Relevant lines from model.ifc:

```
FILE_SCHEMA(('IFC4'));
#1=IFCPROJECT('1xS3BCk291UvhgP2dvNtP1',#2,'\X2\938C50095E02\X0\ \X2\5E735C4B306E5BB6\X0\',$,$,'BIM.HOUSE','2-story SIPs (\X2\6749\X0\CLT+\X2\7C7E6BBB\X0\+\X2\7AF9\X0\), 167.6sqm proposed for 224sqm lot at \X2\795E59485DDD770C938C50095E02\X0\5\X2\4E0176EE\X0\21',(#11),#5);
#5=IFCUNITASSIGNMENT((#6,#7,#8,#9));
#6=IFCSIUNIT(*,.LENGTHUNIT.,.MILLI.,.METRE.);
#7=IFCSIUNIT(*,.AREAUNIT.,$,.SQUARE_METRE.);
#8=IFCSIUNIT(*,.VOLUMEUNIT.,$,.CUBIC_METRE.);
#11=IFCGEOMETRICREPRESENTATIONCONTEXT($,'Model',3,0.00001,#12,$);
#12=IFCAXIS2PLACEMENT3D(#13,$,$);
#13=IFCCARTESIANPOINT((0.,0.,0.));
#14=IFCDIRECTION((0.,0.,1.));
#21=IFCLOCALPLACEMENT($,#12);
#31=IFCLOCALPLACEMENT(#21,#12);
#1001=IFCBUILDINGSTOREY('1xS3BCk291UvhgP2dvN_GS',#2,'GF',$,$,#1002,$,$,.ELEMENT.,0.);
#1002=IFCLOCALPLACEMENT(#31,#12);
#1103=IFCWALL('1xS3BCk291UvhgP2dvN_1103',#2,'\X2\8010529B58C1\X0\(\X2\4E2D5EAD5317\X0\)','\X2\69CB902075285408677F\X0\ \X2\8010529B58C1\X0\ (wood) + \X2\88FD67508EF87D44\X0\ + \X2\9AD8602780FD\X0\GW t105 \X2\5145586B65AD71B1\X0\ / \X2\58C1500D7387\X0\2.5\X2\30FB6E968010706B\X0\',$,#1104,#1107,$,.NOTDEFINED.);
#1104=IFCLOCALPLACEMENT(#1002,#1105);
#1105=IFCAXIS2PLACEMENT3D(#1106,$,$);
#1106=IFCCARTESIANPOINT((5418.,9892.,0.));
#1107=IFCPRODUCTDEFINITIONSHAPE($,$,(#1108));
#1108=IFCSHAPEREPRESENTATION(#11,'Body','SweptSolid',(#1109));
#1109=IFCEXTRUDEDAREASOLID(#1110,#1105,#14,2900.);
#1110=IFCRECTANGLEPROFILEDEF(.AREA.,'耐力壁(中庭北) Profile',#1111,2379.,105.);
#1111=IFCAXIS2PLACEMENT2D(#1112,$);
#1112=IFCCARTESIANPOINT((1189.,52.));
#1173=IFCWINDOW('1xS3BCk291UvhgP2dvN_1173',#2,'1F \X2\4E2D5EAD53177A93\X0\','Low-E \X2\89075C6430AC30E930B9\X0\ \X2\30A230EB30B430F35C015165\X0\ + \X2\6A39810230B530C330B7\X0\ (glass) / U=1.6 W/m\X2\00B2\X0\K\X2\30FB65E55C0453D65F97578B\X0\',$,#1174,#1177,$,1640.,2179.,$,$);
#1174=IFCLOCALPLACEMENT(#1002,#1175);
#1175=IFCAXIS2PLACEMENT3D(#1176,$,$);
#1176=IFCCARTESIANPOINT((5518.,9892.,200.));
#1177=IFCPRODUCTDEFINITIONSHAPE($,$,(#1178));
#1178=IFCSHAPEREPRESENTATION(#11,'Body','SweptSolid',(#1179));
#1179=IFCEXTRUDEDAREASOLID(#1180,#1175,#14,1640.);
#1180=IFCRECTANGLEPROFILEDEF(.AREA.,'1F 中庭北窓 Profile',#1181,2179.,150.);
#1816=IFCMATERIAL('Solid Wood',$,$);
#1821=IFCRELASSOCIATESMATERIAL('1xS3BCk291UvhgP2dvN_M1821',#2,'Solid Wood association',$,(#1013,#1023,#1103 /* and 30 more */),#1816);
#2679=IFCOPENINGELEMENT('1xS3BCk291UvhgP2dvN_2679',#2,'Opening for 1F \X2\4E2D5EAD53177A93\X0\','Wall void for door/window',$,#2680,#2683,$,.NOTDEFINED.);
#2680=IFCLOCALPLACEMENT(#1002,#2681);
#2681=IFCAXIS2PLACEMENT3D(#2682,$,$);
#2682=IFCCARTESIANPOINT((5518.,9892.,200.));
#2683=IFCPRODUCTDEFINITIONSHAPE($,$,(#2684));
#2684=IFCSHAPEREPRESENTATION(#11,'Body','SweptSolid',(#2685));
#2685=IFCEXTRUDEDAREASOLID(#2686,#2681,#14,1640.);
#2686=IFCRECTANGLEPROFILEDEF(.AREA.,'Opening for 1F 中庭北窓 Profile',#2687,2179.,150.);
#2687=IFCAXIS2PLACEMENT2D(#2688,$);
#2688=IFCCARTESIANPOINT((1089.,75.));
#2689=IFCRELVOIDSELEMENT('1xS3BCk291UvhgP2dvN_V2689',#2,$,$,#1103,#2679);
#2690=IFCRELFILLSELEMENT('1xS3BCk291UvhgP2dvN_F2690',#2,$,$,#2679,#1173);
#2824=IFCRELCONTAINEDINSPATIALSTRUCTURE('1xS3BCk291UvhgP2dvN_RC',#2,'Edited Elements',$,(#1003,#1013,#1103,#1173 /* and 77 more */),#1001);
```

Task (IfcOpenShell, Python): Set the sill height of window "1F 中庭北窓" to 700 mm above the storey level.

```python
import numpy as np
import ifcopenshell
import ifcopenshell.api.geometry
import ifcopenshell.geom
import ifcopenshell.util.element
import ifcopenshell.util.placement
import ifcopenshell.util.shape
import ifcopenshell.util.unit

model = ifcopenshell.open("model.ifc")
unit_scale = ifcopenshell.util.unit.calculate_unit_scale(model)

window = model.by_id(1173)
opening = window.FillsVoids[0].RelatingOpeningElement
storey = ifcopenshell.util.element.get_container(window, ifc_class="IfcBuildingStorey")
level = ifcopenshell.util.placement.get_local_placement(storey.ObjectPlacement)[2, 3]

# The opening's origin need not be at the sill, so measure its lowest point.
shape = ifcopenshell.geom.create_shape(ifcopenshell.geom.settings(), opening)
bottom = ifcopenshell.util.shape.get_shape_bottom_elevation(shape, shape.geometry) / unit_scale
dz = level + 700.0 - bottom

shift = np.array([0.0, 0.0, dz])
# The window is not placed relative to its opening, so move both.
for product in (opening, window):
    matrix = ifcopenshell.util.placement.get_local_placement(product.ObjectPlacement)
    matrix[:3, 3] += shift
    ifcopenshell.api.geometry.edit_object_placement(model, product=product, matrix=matrix, is_si=False)

print(f"moved by {dz * unit_scale:+.3f} m")

model.write("model_edited.ifc")
```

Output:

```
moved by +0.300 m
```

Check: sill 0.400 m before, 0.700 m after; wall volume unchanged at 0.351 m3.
